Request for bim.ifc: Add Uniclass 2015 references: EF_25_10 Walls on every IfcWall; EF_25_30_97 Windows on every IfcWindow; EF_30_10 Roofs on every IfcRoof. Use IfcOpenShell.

First a look at what the model holds.

```python
import ifcopenshell

model = ifcopenshell.open("bim.ifc")
print(model.schema)
print("classifications:", [c.Name for c in model.by_type("IfcClassification")])
for ifc_class in ("IfcDoor", "IfcRoof", "IfcStair", "IfcWall", "IfcWindow"):
    print(ifc_class, len(model.by_type(ifc_class)))
```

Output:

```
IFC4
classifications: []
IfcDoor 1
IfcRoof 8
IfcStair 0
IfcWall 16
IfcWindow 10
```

```python
import ifcopenshell
import ifcopenshell.api.classification

model = ifcopenshell.open("bim.ifc")

system = ifcopenshell.api.classification.add_classification(model, classification="Uniclass 2015")

codes = {
    "IfcWall": ("EF_25_10", "Walls"),
    "IfcWindow": ("EF_25_30_97", "Windows"),
    "IfcRoof": ("EF_30_10", "Roofs"),
}
for ifc_class, (code, name) in codes.items():
    products = model.by_type(ifc_class)
    ifcopenshell.api.classification.add_reference(
        model, products=products, classification=system, identification=code, name=name
    )
    print(code, len(products))

model.write("bim_v2.ifc")
```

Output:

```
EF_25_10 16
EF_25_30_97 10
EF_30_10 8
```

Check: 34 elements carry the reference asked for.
